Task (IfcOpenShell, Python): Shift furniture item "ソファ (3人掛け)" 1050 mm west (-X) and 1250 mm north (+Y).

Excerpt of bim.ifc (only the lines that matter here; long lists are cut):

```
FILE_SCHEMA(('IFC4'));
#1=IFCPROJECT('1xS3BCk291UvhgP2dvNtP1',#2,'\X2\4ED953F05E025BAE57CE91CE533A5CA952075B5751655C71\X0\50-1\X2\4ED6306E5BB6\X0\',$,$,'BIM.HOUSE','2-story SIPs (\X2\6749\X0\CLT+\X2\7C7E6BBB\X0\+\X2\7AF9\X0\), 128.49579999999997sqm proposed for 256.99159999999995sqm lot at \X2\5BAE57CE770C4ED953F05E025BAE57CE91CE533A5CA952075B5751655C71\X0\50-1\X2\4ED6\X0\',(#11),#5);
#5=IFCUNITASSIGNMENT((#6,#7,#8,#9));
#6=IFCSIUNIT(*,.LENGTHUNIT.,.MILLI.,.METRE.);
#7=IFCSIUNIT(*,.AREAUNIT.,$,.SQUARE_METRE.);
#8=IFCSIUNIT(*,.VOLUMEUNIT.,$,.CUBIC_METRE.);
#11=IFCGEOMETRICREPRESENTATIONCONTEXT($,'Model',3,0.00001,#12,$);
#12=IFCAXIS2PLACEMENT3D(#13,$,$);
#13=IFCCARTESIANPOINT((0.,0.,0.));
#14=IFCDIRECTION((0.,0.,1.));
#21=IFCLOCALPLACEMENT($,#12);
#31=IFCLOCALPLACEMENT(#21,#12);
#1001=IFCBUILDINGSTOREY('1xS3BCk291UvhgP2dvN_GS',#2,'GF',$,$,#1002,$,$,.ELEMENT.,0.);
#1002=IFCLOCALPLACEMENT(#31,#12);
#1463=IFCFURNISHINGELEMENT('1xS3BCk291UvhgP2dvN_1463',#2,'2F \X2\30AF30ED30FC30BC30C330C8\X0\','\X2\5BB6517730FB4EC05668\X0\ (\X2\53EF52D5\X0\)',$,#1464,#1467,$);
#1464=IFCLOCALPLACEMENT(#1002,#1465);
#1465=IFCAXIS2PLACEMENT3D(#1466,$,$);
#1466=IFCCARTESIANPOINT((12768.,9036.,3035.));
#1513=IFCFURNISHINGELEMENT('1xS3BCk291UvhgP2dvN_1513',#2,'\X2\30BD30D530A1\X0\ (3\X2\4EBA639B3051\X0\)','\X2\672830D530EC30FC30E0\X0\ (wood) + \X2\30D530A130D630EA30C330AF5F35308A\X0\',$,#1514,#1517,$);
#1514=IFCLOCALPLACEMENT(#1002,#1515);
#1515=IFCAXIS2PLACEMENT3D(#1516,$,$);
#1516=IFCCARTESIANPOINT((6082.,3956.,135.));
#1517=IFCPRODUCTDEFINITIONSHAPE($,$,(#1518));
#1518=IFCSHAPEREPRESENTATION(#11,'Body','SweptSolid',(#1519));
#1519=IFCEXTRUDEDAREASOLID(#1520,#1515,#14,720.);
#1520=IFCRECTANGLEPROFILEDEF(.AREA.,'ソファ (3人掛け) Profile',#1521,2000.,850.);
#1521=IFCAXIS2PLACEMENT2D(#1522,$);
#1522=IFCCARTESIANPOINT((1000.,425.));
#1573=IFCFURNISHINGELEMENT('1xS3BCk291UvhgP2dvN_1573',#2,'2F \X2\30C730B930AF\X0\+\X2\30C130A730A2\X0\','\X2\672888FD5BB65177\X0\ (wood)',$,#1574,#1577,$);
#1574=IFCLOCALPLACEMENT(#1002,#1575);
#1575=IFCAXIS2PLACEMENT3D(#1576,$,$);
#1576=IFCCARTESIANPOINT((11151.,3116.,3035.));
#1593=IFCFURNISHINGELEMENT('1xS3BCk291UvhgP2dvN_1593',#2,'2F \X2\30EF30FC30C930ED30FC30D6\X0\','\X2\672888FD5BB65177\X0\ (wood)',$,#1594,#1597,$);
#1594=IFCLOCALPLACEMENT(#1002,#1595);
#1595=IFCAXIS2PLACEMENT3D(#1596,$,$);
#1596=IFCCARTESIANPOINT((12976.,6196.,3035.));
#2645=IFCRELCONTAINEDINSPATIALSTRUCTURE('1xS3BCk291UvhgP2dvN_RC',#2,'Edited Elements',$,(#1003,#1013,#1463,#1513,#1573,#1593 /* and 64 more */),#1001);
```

```python
import ifcopenshell
import ifcopenshell.api.geometry
import ifcopenshell.util.placement
import ifcopenshell.util.unit

model = ifcopenshell.open("bim.ifc")
unit_scale = ifcopenshell.util.unit.calculate_unit_scale(model)

item = model.by_id(1513)
matrix = ifcopenshell.util.placement.get_local_placement(item.ObjectPlacement)
matrix[0, 3] -= 1.05 / unit_scale
matrix[1, 3] += 1.25 / unit_scale
ifcopenshell.api.geometry.edit_object_placement(model, product=item, matrix=matrix, is_si=False)

print(ifcopenshell.util.placement.get_local_placement(item.ObjectPlacement).round(3) + 0.0)

model.write("bim-out.ifc")
```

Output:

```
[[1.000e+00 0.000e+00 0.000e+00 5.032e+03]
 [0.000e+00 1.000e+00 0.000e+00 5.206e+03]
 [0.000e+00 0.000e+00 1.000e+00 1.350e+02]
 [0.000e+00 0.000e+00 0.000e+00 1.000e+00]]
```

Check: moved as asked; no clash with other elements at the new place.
